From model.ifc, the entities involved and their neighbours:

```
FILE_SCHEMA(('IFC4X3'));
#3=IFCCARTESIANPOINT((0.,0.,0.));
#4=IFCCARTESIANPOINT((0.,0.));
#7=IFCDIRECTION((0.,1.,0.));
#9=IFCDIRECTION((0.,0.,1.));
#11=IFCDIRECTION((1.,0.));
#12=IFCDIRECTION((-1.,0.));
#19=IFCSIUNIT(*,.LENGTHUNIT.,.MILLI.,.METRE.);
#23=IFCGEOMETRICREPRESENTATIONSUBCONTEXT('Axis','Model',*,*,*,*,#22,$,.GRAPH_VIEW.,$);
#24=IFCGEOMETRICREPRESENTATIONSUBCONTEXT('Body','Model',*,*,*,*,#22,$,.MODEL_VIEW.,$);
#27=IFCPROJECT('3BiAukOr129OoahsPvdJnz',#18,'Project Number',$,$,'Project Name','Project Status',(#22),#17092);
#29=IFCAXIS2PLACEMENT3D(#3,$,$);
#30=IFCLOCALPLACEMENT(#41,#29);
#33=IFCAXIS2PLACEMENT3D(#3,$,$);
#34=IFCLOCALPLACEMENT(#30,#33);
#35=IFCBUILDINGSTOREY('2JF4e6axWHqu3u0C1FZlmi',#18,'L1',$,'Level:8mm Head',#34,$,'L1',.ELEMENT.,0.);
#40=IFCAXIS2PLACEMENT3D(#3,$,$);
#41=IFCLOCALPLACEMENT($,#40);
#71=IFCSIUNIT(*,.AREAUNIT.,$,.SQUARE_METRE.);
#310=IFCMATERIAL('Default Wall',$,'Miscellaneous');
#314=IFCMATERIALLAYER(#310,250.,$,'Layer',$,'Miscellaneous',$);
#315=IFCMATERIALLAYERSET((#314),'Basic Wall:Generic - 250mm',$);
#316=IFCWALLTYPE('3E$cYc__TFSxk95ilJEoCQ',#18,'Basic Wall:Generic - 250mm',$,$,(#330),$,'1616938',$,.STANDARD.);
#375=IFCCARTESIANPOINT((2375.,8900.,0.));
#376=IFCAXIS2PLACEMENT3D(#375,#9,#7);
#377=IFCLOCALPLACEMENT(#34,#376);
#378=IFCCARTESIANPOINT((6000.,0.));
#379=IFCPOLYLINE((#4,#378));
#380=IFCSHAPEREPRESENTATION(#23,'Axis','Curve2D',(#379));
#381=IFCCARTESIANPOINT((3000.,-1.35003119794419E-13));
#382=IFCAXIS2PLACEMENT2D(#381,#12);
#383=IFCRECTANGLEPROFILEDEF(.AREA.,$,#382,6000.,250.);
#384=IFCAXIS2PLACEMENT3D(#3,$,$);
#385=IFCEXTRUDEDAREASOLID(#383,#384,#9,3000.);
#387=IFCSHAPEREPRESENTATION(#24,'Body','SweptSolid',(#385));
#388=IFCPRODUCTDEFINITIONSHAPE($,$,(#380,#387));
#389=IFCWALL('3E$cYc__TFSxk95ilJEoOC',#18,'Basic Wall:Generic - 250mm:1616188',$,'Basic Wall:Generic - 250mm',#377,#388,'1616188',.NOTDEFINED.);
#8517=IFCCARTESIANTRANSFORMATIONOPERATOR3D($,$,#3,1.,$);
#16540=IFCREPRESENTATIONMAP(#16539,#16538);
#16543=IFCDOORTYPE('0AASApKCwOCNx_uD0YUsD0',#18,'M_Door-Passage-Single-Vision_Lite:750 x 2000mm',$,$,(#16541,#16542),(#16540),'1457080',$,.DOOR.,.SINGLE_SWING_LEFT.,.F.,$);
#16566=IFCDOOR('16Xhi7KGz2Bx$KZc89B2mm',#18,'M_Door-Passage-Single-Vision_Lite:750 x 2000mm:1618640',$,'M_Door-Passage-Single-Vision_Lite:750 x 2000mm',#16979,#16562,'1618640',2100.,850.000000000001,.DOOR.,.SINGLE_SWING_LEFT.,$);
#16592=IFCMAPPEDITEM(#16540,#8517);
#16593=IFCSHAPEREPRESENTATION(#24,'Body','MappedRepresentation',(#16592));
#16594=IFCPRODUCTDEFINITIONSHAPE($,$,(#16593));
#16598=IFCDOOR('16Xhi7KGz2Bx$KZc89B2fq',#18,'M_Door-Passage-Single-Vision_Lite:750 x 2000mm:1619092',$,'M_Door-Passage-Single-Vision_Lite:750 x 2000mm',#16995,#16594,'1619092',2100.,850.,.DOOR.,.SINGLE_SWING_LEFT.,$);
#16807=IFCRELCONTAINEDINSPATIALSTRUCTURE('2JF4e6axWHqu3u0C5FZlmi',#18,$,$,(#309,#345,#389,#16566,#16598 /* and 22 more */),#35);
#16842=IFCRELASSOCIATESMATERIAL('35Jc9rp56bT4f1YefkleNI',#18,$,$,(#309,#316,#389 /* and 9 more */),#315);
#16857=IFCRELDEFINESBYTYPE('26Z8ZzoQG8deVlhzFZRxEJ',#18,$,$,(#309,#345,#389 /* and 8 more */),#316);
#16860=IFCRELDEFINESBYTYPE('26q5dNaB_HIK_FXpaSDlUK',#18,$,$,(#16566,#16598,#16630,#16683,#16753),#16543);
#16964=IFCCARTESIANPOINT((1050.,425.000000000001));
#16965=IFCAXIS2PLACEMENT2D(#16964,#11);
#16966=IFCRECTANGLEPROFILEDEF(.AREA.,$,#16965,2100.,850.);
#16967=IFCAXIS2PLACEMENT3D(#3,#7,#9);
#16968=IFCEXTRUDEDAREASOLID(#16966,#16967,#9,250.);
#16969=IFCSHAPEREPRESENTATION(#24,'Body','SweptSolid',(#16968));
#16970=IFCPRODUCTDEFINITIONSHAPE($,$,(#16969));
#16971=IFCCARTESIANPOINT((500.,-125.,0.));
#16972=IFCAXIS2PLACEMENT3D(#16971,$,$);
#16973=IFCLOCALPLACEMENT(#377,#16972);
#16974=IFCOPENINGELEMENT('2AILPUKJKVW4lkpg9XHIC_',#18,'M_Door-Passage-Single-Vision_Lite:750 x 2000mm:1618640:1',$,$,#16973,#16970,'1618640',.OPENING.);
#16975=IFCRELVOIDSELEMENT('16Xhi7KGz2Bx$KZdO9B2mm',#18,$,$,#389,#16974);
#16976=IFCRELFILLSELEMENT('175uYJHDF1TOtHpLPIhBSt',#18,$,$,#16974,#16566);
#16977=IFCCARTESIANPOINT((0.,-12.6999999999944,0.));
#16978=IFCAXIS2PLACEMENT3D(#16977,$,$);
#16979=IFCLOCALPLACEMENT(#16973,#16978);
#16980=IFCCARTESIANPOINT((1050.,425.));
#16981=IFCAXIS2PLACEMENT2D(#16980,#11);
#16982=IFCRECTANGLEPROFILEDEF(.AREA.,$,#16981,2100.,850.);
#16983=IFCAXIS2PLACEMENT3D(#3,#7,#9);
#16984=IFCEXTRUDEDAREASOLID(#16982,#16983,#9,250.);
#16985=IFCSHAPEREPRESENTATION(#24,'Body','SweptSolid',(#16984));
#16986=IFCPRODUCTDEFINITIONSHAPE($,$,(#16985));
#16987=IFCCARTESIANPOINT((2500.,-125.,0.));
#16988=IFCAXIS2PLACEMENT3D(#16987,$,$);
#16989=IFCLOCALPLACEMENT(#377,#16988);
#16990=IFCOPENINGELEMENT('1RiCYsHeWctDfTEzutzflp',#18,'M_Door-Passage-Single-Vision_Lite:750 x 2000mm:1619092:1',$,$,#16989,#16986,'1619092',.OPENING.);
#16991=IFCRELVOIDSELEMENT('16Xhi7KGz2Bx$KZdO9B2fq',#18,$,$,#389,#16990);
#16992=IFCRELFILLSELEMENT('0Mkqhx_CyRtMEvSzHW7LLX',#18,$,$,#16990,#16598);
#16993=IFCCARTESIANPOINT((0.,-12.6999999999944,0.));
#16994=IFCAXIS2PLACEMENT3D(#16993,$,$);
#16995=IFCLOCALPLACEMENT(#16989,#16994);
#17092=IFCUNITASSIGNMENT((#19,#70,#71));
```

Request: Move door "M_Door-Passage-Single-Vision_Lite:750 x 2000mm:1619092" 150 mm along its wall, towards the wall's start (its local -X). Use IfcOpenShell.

```python
import ifcopenshell
import ifcopenshell.api.geometry
import ifcopenshell.util.placement
import ifcopenshell.util.unit

model = ifcopenshell.open("model.ifc")
unit_scale = ifcopenshell.util.unit.calculate_unit_scale(model)

door = model.by_id(16598)
opening = door.FillsVoids[0].RelatingOpeningElement
wall = opening.VoidsElements[0].RelatingBuildingElement

wall_matrix = ifcopenshell.util.placement.get_local_placement(wall.ObjectPlacement)
shift = wall_matrix[:3, 0] * -0.15 / unit_scale
before = ifcopenshell.util.placement.get_local_placement(door.ObjectPlacement)[:3, 3].copy()

# The door is placed relative to its opening, so it follows when the opening moves.
matrix = ifcopenshell.util.placement.get_local_placement(opening.ObjectPlacement)
matrix[:3, 3] += shift
ifcopenshell.api.geometry.edit_object_placement(
    model, product=opening, matrix=matrix, is_si=False, should_transform_children=True
)

after = ifcopenshell.util.placement.get_local_placement(door.ObjectPlacement)[:3, 3]
print("door moved by", (after - before).round(3) + 0.0)

model.write("model_v2.ifc")
```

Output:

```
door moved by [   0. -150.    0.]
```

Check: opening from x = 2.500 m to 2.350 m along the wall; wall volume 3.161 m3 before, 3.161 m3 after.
